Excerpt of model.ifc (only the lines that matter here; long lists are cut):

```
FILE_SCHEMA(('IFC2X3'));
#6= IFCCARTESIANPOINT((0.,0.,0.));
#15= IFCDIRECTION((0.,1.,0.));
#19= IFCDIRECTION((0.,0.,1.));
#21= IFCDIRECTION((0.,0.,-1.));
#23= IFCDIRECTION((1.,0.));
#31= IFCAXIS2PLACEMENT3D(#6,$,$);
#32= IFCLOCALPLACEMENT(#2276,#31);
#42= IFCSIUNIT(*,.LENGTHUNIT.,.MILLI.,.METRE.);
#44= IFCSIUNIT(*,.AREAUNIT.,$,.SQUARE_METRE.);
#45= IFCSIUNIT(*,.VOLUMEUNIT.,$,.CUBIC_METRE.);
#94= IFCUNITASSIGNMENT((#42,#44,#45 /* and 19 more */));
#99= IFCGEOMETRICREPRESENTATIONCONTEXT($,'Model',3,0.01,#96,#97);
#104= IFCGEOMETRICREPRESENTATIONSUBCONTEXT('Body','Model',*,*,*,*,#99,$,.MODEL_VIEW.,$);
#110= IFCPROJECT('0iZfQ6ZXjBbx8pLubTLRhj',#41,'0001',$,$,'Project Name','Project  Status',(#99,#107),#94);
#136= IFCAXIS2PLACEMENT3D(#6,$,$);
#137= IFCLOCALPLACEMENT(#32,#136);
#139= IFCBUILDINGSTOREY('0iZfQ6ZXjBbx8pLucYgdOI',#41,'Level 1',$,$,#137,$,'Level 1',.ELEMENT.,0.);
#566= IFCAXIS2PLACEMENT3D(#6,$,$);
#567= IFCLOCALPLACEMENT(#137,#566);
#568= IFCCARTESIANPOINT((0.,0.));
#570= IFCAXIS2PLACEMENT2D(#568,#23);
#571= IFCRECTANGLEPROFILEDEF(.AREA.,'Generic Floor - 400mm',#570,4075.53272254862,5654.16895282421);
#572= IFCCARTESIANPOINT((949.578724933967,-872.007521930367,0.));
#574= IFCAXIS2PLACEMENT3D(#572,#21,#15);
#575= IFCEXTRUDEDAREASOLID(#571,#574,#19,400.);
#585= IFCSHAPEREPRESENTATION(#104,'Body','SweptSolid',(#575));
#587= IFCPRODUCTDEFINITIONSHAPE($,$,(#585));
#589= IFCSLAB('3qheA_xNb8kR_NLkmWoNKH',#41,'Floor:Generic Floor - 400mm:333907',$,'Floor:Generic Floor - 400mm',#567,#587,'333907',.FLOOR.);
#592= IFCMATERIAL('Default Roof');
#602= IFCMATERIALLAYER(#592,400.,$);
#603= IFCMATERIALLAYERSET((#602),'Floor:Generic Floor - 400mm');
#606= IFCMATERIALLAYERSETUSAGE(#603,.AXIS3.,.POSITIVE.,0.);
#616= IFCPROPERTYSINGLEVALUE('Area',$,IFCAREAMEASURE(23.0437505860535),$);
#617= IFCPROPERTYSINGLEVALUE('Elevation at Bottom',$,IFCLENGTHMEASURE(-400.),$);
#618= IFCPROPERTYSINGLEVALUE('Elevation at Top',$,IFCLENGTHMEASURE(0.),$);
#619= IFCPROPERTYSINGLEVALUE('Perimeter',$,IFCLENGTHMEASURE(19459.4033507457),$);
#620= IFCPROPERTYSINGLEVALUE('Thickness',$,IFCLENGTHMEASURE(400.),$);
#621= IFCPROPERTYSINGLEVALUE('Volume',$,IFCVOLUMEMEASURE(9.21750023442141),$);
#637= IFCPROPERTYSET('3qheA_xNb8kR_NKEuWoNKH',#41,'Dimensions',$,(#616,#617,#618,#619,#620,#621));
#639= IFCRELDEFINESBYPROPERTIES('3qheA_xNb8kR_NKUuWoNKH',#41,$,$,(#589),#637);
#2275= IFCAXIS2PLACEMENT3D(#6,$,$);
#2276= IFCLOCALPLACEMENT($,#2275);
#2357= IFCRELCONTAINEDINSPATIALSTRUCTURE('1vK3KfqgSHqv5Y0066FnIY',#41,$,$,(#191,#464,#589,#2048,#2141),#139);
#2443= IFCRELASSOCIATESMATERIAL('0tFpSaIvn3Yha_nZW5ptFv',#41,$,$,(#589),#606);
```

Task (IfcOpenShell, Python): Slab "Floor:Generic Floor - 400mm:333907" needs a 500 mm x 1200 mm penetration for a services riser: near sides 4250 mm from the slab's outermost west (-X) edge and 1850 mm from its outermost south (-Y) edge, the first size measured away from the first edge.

```python
import numpy as np
import ifcopenshell
import ifcopenshell.api.feature
import ifcopenshell.api.geometry
import ifcopenshell.api.pset
import ifcopenshell.api.root
import ifcopenshell.geom
import ifcopenshell.util.element
import ifcopenshell.util.placement
import ifcopenshell.util.representation
import ifcopenshell.util.shape
import ifcopenshell.util.unit

model = ifcopenshell.open("model.ifc")
unit_scale = ifcopenshell.util.unit.calculate_unit_scale(model)
area_scale = ifcopenshell.util.unit.calculate_unit_scale(model, "AREAUNIT")
volume_scale = ifcopenshell.util.unit.calculate_unit_scale(model, "VOLUMEUNIT")
settings = ifcopenshell.geom.settings()


def volume(element):
    """Net volume in cubic metres, openings subtracted."""
    shape = ifcopenshell.geom.create_shape(settings, element)
    return ifcopenshell.util.shape.get_volume(shape.geometry)


slab = model.by_guid("3qheA_xNb8kR_NLkmWoNKH")
before = volume(slab)

# Extent in the slab's own axes, in metres. The edges named are its -X and -Y sides.
slab_shape = ifcopenshell.geom.create_shape(settings, slab)
vertices = ifcopenshell.util.shape.get_vertices(slab_shape.geometry)
x_min, y_min, bottom = vertices.min(axis=0)
top = vertices[:, 2].max()

opening = ifcopenshell.api.root.create_entity(model, ifc_class="IfcOpeningElement", name="Services riser opening")
context = ifcopenshell.util.representation.get_context(model, "Model", "Body", "MODEL_VIEW")
width, depth = 0.5, 1.2
outline = [(0.0, 0.0), (width, 0.0), (width, depth), (0.0, depth), (0.0, 0.0)]
# Overshoot both faces by 50 mm so the cut is clean.
shape = ifcopenshell.api.geometry.add_slab_representation(
    model, context=context, depth=top - bottom + 0.1, polyline=outline
)
ifcopenshell.api.geometry.assign_representation(model, product=opening, representation=shape)

matrix = ifcopenshell.util.placement.get_local_placement(slab.ObjectPlacement)
matrix[:, 3] = matrix @ np.append(np.array([x_min + 4.25, y_min + 1.85, bottom - 0.05]) / unit_scale, 1.0)
ifcopenshell.api.geometry.edit_object_placement(model, product=opening, matrix=matrix, is_si=False)
ifcopenshell.api.feature.add_feature(model, feature=opening, element=slab)

after = volume(slab)

# Update the slab's stored quantities.
pset = model.by_id(ifcopenshell.util.element.get_pset(slab, "Dimensions", should_inherit=False)["id"])
ifcopenshell.api.pset.edit_pset(model, pset=pset, properties={
    "Area": model.create_entity("IfcAreaMeasure", after / (top - bottom) / area_scale),
    "Volume": model.create_entity("IfcVolumeMeasure", after / volume_scale),
})

print(f"slab volume {before:.3f} -> {after:.3f} m3")

model.write("model_rev.ifc")
```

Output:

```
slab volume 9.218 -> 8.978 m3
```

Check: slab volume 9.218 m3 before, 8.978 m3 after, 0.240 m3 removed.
